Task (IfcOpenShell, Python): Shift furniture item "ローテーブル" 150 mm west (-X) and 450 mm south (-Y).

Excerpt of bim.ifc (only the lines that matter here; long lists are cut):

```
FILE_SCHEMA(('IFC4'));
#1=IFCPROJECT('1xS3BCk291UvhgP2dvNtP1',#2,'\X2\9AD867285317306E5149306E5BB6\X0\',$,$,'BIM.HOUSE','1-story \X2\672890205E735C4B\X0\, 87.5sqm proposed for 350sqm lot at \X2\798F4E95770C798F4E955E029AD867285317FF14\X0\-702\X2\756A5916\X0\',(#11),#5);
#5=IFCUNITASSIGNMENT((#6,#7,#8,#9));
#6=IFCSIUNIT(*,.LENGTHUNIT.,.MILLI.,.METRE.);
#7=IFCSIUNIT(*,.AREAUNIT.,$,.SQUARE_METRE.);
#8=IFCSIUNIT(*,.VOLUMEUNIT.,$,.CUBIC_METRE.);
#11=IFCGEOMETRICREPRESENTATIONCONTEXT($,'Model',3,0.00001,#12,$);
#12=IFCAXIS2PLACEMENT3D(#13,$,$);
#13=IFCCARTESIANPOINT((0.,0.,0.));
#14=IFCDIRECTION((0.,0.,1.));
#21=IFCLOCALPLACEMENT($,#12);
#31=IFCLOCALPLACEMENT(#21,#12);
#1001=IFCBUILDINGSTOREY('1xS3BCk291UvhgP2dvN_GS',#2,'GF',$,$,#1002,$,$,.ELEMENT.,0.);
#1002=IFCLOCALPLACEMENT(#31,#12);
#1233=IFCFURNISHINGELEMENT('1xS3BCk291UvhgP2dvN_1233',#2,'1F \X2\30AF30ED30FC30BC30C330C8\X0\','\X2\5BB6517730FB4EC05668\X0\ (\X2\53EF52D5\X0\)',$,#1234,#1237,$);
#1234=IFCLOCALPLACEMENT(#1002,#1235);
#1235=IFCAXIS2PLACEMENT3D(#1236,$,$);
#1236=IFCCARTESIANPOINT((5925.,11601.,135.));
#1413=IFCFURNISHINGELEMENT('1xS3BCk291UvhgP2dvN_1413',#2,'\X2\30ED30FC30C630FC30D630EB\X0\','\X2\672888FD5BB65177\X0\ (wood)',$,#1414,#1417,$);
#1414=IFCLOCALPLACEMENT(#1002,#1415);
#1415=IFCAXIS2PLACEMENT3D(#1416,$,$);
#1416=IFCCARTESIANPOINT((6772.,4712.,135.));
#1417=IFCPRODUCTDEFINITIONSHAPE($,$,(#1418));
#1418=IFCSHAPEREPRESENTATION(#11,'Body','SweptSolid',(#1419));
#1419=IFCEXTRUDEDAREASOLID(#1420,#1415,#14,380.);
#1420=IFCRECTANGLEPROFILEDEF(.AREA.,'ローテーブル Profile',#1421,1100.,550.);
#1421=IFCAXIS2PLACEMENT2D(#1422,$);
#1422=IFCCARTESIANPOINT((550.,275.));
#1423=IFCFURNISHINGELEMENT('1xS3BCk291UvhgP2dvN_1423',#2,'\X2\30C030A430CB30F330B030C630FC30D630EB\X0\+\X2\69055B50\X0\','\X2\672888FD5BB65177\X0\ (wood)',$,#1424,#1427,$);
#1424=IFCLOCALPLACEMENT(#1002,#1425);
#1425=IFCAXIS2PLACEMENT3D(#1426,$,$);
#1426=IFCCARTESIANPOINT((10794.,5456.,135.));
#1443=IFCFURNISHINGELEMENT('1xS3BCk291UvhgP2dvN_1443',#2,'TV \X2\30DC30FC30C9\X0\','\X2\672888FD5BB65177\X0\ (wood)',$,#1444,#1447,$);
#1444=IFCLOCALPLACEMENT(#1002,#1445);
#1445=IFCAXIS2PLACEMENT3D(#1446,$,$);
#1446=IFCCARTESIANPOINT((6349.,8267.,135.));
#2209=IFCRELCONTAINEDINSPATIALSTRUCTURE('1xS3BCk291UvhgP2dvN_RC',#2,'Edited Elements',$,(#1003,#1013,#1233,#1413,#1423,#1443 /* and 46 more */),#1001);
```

```python
import ifcopenshell
import ifcopenshell.api.geometry
import ifcopenshell.util.placement
import ifcopenshell.util.unit

model = ifcopenshell.open("bim.ifc")
unit_scale = ifcopenshell.util.unit.calculate_unit_scale(model)

item = model.by_id(1413)
matrix = ifcopenshell.util.placement.get_local_placement(item.ObjectPlacement)
matrix[0, 3] -= 0.15 / unit_scale
matrix[1, 3] -= 0.45 / unit_scale
ifcopenshell.api.geometry.edit_object_placement(model, product=item, matrix=matrix, is_si=False)

print(ifcopenshell.util.placement.get_local_placement(item.ObjectPlacement).round(3) + 0.0)

model.write("bim_edited.ifc")
```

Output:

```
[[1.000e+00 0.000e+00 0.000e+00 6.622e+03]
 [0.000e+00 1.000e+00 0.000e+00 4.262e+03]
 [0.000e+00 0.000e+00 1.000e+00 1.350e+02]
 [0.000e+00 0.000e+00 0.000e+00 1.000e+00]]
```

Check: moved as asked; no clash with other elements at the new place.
